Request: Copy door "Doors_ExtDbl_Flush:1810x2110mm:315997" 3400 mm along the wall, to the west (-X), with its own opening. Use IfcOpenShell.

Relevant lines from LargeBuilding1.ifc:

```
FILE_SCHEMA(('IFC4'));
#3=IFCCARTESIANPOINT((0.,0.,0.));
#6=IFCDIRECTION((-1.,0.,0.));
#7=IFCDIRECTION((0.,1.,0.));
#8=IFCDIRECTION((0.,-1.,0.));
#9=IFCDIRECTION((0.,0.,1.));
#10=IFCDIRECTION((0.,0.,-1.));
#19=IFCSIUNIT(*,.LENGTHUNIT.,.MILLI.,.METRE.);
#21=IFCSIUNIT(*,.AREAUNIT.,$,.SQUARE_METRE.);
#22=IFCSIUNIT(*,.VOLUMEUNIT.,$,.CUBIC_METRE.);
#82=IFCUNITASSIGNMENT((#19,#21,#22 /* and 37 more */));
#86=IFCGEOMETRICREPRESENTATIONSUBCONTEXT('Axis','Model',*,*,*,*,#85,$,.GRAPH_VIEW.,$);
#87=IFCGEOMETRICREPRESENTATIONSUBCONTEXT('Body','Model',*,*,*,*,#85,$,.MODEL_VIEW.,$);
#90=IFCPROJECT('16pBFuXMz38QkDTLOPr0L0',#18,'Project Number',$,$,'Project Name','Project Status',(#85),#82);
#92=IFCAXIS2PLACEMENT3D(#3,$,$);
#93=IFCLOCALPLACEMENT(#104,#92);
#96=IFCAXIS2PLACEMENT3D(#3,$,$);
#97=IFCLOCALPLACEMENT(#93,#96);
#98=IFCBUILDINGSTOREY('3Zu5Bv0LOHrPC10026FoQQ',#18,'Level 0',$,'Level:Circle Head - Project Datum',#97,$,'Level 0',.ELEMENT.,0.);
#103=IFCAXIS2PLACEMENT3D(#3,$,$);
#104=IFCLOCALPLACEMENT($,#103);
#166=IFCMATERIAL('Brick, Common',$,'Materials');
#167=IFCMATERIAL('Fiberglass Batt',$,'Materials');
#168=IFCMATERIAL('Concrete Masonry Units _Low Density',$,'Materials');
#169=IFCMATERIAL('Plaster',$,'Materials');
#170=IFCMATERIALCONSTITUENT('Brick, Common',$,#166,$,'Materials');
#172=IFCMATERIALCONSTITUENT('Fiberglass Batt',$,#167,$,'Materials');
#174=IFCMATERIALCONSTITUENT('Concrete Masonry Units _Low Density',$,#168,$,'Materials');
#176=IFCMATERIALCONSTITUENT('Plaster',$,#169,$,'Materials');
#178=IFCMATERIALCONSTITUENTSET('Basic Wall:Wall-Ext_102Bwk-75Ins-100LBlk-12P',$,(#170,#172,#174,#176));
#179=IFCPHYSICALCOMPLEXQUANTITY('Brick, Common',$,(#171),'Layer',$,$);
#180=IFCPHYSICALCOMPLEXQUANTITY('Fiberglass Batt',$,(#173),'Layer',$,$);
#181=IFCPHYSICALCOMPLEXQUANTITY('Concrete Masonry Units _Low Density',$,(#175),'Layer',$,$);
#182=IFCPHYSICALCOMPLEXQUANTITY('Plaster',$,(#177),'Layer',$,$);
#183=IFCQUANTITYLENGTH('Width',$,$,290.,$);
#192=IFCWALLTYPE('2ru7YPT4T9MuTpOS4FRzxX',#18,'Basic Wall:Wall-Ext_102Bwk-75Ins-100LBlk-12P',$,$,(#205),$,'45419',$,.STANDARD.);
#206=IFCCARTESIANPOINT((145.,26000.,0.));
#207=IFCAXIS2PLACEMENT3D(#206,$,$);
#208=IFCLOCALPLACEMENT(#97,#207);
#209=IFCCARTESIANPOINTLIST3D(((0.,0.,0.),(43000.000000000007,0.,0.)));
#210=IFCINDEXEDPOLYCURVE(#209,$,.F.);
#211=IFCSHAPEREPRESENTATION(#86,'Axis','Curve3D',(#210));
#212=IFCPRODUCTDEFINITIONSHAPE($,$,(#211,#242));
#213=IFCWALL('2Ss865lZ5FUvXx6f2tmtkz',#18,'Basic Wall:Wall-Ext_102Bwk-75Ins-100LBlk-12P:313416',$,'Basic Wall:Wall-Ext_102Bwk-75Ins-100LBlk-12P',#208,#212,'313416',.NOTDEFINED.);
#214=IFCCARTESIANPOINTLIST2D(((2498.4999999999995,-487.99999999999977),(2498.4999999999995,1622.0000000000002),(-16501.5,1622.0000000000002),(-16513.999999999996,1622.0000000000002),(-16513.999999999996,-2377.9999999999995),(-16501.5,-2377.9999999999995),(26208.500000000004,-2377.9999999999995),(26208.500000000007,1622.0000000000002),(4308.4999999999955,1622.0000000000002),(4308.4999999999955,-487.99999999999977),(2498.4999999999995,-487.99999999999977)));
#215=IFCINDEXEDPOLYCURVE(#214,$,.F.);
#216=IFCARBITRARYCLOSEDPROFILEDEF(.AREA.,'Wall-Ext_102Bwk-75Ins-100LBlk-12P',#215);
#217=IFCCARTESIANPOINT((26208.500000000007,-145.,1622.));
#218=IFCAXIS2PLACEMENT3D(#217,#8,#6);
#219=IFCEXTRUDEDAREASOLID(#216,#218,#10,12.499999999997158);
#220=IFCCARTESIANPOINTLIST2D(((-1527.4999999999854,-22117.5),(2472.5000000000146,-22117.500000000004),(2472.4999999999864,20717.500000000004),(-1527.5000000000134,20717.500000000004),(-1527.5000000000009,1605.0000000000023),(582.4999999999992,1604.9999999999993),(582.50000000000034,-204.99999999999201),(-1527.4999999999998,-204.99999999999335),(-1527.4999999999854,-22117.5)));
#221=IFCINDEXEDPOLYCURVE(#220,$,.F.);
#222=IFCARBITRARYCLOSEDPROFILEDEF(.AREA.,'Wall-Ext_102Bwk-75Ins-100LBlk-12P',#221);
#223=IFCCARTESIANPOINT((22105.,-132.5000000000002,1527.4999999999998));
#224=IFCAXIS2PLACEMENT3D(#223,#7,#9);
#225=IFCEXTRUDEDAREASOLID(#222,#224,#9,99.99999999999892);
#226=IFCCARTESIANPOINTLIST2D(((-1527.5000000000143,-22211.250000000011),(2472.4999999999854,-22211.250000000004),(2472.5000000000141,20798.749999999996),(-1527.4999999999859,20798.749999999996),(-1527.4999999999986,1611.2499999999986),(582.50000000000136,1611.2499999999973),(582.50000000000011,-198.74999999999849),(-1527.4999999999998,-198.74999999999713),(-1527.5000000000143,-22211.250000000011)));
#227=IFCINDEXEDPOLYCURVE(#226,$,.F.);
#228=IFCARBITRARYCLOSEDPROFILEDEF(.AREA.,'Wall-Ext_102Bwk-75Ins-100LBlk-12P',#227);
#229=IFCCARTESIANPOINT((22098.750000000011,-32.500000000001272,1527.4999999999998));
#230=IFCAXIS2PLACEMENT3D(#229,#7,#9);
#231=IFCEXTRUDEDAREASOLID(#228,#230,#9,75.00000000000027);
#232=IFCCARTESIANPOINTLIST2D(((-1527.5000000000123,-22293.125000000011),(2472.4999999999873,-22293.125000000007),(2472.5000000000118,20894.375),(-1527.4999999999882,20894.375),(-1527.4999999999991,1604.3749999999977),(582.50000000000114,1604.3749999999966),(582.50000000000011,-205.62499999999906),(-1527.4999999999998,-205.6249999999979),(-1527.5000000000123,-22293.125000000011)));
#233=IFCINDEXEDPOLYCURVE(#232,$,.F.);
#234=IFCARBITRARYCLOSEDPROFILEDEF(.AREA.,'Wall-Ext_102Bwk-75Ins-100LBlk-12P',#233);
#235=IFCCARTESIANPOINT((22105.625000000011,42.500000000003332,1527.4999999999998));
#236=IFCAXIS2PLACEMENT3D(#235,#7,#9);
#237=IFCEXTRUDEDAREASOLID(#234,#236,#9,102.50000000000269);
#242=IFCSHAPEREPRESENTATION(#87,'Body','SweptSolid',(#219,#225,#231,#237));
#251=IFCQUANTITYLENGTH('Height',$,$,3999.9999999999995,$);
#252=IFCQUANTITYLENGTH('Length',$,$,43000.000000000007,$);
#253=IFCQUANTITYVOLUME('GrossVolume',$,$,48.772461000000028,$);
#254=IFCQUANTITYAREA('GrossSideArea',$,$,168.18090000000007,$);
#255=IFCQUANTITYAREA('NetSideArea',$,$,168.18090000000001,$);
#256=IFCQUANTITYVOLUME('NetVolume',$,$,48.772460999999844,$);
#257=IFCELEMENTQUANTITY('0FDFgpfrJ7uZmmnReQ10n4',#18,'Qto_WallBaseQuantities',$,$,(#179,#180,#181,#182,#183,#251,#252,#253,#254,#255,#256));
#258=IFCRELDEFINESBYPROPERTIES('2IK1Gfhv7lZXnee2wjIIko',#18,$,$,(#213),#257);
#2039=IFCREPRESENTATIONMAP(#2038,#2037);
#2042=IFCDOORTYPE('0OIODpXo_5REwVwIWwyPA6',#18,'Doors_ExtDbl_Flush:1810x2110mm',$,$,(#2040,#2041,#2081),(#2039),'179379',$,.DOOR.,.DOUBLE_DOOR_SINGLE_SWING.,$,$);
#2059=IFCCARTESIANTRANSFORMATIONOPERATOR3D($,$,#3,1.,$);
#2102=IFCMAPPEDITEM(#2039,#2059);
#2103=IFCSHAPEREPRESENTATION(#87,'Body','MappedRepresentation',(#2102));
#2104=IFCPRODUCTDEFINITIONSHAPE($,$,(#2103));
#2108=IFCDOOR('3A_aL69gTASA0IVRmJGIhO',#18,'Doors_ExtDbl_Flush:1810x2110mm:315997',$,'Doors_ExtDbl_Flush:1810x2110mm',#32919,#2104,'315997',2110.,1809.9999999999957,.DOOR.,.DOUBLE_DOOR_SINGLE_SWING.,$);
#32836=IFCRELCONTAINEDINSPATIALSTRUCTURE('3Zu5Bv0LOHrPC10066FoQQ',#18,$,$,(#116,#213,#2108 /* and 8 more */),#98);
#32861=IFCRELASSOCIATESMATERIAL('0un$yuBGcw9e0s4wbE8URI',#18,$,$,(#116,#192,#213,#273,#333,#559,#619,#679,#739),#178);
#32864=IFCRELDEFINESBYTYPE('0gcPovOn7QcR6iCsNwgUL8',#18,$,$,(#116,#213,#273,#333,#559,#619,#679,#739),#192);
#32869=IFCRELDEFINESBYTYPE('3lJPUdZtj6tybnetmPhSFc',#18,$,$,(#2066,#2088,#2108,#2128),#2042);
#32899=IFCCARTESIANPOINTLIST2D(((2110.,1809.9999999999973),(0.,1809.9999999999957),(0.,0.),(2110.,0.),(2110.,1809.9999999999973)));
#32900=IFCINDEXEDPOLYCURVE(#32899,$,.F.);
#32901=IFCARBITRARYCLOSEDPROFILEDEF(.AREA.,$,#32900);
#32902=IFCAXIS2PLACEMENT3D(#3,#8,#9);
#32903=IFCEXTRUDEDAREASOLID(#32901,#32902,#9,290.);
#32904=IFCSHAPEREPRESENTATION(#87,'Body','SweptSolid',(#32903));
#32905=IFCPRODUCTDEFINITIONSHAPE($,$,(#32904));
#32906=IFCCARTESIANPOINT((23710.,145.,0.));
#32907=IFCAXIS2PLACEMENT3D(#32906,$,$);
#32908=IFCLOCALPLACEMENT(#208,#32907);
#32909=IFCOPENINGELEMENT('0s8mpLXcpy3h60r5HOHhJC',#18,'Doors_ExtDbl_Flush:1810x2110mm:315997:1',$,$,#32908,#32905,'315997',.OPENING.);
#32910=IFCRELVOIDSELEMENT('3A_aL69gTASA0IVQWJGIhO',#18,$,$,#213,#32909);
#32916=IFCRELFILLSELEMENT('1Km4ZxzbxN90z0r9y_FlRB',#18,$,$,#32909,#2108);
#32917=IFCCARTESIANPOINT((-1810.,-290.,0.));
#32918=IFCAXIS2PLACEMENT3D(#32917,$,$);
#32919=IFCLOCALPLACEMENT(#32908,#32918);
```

```python
import ifcopenshell
import ifcopenshell.api.feature
import ifcopenshell.api.geometry
import ifcopenshell.api.pset
import ifcopenshell.api.root
import ifcopenshell.geom
import ifcopenshell.util.element
import ifcopenshell.util.placement
import ifcopenshell.util.shape
import ifcopenshell.util.unit

model = ifcopenshell.open("LargeBuilding1.ifc")
unit_scale = ifcopenshell.util.unit.calculate_unit_scale(model)
area_scale = ifcopenshell.util.unit.calculate_unit_scale(model, "AREAUNIT")
volume_scale = ifcopenshell.util.unit.calculate_unit_scale(model, "VOLUMEUNIT")
settings = ifcopenshell.geom.settings()


def volume(element):
    """Net volume in cubic metres, openings subtracted."""
    shape = ifcopenshell.geom.create_shape(settings, element)
    return ifcopenshell.util.shape.get_volume(shape.geometry)


def reuse_history(source, copy):
    """copy_class also copies each property set's owner history, people and application; keep the originals."""
    for rel in copy.IsDefinedBy:
        if rel.is_a("IfcRelDefinesByProperties") and (history := rel.RelatingPropertyDefinition.OwnerHistory):
            rel.RelatingPropertyDefinition.OwnerHistory = source.OwnerHistory
            ifcopenshell.util.element.remove_deep2(model, history)


door = model.by_guid("3A_aL69gTASA0IVRmJGIhO")
opening = door.FillsVoids[0].RelatingOpeningElement
wall = opening.VoidsElements[0].RelatingBuildingElement
before = volume(wall)
shift = ifcopenshell.util.placement.get_local_placement(wall.ObjectPlacement)[:3, 0] * -3.4 / unit_scale

# copy_class copies the void relationship, type, container and properties, but no geometry.
new_opening = ifcopenshell.api.root.copy_class(model, product=opening)
new_opening.Representation = ifcopenshell.util.element.copy_deep(
    model, opening.Representation, exclude=["IfcGeometricRepresentationContext", "IfcRepresentationMap"]
)
new_opening.Name = "Doors_ExtDbl_Flush:1810x2110mm"
new_opening.Tag = None
reuse_history(opening, new_opening)
new_door = ifcopenshell.api.root.copy_class(model, product=door)
new_door.Representation = ifcopenshell.util.element.copy_deep(
    model, door.Representation, exclude=["IfcGeometricRepresentationContext", "IfcRepresentationMap"]
)
new_door.Name = "Doors_ExtDbl_Flush:1810x2110mm"
new_door.Tag = None
reuse_history(door, new_door)
ifcopenshell.api.feature.add_filling(model, opening=new_opening, element=new_door)

for old, new in ((opening, new_opening), (door, new_door)):
    matrix = ifcopenshell.util.placement.get_local_placement(old.ObjectPlacement)
    matrix[:3, 3] += shift
    ifcopenshell.api.geometry.edit_object_placement(model, product=new, matrix=matrix, is_si=False)

after = volume(wall)
thickness = 0.29  # wall thickness in metres

# Update the wall's stored quantities.
qto = model.by_id(ifcopenshell.util.element.get_pset(wall, "Qto_WallBaseQuantities", should_inherit=False)["id"])
ifcopenshell.api.pset.edit_qto(model, qto=qto, properties={
    "NetSideArea": after / thickness / area_scale,
    "NetVolume": after / volume_scale,
})

print(f"wall volume {before:.3f} -> {after:.3f} m3")

model.write("LargeBuilding1_v2.ifc")
```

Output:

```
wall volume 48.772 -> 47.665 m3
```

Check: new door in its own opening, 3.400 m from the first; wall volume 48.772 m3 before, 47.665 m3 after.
